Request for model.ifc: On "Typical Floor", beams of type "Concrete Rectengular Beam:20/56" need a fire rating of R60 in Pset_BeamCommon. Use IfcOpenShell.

First a look at what the model holds.

```python
import ifcopenshell
import ifcopenshell.util.element

model = ifcopenshell.open("model.ifc")
print(model.schema)
storey = next(s for s in model.by_type("IfcBuildingStorey") if s.Name == "Typical Floor")
beams = [e for e in ifcopenshell.util.element.get_decomposition(storey) if e.is_a("IfcBeam")]
seen = {}
for e in beams:
    element_type = ifcopenshell.util.element.get_type(e)
    key = (element_type.Name if element_type != e and element_type else None, ifcopenshell.util.element.get_pset(e, "Pset_BeamCommon", "FireRating"))
    seen[key] = seen.get(key, 0) + 1
for (name, value), count in sorted(seen.items(), key=str):
    print(count, "x", name, "|", value)
```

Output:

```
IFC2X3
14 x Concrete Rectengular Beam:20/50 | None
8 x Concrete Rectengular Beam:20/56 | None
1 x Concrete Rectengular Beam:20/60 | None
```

```python
import ifcopenshell
import ifcopenshell.api.pset
import ifcopenshell.util.element

model = ifcopenshell.open("model.ifc")

storey = next(s for s in model.by_type("IfcBuildingStorey") if s.Name == "Typical Floor")
beams = [e for e in ifcopenshell.util.element.get_decomposition(storey) if e.is_a("IfcBeam")]

count = 0
for e in beams:
    element_type = ifcopenshell.util.element.get_type(e)
    if element_type in (None, e) or element_type.Name != "Concrete Rectengular Beam:20/56":
        continue
    # add_pset returns the element's existing set when there is one.
    pset = ifcopenshell.api.pset.add_pset(model, product=e, name="Pset_BeamCommon")
    ifcopenshell.api.pset.edit_pset(model, pset=pset, properties={"FireRating": "R60"})
    count += 1

print(count, "beams updated")

model.write("model_v2.ifc")
```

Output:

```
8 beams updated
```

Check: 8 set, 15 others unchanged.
